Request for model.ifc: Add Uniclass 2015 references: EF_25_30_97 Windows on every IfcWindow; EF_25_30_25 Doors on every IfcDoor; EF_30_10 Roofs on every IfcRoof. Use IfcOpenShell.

First a look at what the model holds.

```python
import ifcopenshell

model = ifcopenshell.open("model.ifc")
print(model.schema)
print("classifications:", [c.Name for c in model.by_type("IfcClassification")])
for ifc_class in ("IfcDoor", "IfcRoof", "IfcStair", "IfcWall", "IfcWindow"):
    print(ifc_class, len(model.by_type(ifc_class)))
```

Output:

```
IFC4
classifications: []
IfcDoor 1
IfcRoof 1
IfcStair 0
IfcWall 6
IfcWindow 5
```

```python
import ifcopenshell
import ifcopenshell.api.classification

model = ifcopenshell.open("model.ifc")

system = ifcopenshell.api.classification.add_classification(model, classification="Uniclass 2015")

codes = {
    "IfcWindow": ("EF_25_30_97", "Windows"),
    "IfcDoor": ("EF_25_30_25", "Doors"),
    "IfcRoof": ("EF_30_10", "Roofs"),
}
for ifc_class, (code, name) in codes.items():
    products = model.by_type(ifc_class)
    ifcopenshell.api.classification.add_reference(
        model, products=products, classification=system, identification=code, name=name
    )
    print(code, len(products))

model.write("model_updated.ifc")
```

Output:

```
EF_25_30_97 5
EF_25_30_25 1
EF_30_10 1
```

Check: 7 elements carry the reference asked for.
